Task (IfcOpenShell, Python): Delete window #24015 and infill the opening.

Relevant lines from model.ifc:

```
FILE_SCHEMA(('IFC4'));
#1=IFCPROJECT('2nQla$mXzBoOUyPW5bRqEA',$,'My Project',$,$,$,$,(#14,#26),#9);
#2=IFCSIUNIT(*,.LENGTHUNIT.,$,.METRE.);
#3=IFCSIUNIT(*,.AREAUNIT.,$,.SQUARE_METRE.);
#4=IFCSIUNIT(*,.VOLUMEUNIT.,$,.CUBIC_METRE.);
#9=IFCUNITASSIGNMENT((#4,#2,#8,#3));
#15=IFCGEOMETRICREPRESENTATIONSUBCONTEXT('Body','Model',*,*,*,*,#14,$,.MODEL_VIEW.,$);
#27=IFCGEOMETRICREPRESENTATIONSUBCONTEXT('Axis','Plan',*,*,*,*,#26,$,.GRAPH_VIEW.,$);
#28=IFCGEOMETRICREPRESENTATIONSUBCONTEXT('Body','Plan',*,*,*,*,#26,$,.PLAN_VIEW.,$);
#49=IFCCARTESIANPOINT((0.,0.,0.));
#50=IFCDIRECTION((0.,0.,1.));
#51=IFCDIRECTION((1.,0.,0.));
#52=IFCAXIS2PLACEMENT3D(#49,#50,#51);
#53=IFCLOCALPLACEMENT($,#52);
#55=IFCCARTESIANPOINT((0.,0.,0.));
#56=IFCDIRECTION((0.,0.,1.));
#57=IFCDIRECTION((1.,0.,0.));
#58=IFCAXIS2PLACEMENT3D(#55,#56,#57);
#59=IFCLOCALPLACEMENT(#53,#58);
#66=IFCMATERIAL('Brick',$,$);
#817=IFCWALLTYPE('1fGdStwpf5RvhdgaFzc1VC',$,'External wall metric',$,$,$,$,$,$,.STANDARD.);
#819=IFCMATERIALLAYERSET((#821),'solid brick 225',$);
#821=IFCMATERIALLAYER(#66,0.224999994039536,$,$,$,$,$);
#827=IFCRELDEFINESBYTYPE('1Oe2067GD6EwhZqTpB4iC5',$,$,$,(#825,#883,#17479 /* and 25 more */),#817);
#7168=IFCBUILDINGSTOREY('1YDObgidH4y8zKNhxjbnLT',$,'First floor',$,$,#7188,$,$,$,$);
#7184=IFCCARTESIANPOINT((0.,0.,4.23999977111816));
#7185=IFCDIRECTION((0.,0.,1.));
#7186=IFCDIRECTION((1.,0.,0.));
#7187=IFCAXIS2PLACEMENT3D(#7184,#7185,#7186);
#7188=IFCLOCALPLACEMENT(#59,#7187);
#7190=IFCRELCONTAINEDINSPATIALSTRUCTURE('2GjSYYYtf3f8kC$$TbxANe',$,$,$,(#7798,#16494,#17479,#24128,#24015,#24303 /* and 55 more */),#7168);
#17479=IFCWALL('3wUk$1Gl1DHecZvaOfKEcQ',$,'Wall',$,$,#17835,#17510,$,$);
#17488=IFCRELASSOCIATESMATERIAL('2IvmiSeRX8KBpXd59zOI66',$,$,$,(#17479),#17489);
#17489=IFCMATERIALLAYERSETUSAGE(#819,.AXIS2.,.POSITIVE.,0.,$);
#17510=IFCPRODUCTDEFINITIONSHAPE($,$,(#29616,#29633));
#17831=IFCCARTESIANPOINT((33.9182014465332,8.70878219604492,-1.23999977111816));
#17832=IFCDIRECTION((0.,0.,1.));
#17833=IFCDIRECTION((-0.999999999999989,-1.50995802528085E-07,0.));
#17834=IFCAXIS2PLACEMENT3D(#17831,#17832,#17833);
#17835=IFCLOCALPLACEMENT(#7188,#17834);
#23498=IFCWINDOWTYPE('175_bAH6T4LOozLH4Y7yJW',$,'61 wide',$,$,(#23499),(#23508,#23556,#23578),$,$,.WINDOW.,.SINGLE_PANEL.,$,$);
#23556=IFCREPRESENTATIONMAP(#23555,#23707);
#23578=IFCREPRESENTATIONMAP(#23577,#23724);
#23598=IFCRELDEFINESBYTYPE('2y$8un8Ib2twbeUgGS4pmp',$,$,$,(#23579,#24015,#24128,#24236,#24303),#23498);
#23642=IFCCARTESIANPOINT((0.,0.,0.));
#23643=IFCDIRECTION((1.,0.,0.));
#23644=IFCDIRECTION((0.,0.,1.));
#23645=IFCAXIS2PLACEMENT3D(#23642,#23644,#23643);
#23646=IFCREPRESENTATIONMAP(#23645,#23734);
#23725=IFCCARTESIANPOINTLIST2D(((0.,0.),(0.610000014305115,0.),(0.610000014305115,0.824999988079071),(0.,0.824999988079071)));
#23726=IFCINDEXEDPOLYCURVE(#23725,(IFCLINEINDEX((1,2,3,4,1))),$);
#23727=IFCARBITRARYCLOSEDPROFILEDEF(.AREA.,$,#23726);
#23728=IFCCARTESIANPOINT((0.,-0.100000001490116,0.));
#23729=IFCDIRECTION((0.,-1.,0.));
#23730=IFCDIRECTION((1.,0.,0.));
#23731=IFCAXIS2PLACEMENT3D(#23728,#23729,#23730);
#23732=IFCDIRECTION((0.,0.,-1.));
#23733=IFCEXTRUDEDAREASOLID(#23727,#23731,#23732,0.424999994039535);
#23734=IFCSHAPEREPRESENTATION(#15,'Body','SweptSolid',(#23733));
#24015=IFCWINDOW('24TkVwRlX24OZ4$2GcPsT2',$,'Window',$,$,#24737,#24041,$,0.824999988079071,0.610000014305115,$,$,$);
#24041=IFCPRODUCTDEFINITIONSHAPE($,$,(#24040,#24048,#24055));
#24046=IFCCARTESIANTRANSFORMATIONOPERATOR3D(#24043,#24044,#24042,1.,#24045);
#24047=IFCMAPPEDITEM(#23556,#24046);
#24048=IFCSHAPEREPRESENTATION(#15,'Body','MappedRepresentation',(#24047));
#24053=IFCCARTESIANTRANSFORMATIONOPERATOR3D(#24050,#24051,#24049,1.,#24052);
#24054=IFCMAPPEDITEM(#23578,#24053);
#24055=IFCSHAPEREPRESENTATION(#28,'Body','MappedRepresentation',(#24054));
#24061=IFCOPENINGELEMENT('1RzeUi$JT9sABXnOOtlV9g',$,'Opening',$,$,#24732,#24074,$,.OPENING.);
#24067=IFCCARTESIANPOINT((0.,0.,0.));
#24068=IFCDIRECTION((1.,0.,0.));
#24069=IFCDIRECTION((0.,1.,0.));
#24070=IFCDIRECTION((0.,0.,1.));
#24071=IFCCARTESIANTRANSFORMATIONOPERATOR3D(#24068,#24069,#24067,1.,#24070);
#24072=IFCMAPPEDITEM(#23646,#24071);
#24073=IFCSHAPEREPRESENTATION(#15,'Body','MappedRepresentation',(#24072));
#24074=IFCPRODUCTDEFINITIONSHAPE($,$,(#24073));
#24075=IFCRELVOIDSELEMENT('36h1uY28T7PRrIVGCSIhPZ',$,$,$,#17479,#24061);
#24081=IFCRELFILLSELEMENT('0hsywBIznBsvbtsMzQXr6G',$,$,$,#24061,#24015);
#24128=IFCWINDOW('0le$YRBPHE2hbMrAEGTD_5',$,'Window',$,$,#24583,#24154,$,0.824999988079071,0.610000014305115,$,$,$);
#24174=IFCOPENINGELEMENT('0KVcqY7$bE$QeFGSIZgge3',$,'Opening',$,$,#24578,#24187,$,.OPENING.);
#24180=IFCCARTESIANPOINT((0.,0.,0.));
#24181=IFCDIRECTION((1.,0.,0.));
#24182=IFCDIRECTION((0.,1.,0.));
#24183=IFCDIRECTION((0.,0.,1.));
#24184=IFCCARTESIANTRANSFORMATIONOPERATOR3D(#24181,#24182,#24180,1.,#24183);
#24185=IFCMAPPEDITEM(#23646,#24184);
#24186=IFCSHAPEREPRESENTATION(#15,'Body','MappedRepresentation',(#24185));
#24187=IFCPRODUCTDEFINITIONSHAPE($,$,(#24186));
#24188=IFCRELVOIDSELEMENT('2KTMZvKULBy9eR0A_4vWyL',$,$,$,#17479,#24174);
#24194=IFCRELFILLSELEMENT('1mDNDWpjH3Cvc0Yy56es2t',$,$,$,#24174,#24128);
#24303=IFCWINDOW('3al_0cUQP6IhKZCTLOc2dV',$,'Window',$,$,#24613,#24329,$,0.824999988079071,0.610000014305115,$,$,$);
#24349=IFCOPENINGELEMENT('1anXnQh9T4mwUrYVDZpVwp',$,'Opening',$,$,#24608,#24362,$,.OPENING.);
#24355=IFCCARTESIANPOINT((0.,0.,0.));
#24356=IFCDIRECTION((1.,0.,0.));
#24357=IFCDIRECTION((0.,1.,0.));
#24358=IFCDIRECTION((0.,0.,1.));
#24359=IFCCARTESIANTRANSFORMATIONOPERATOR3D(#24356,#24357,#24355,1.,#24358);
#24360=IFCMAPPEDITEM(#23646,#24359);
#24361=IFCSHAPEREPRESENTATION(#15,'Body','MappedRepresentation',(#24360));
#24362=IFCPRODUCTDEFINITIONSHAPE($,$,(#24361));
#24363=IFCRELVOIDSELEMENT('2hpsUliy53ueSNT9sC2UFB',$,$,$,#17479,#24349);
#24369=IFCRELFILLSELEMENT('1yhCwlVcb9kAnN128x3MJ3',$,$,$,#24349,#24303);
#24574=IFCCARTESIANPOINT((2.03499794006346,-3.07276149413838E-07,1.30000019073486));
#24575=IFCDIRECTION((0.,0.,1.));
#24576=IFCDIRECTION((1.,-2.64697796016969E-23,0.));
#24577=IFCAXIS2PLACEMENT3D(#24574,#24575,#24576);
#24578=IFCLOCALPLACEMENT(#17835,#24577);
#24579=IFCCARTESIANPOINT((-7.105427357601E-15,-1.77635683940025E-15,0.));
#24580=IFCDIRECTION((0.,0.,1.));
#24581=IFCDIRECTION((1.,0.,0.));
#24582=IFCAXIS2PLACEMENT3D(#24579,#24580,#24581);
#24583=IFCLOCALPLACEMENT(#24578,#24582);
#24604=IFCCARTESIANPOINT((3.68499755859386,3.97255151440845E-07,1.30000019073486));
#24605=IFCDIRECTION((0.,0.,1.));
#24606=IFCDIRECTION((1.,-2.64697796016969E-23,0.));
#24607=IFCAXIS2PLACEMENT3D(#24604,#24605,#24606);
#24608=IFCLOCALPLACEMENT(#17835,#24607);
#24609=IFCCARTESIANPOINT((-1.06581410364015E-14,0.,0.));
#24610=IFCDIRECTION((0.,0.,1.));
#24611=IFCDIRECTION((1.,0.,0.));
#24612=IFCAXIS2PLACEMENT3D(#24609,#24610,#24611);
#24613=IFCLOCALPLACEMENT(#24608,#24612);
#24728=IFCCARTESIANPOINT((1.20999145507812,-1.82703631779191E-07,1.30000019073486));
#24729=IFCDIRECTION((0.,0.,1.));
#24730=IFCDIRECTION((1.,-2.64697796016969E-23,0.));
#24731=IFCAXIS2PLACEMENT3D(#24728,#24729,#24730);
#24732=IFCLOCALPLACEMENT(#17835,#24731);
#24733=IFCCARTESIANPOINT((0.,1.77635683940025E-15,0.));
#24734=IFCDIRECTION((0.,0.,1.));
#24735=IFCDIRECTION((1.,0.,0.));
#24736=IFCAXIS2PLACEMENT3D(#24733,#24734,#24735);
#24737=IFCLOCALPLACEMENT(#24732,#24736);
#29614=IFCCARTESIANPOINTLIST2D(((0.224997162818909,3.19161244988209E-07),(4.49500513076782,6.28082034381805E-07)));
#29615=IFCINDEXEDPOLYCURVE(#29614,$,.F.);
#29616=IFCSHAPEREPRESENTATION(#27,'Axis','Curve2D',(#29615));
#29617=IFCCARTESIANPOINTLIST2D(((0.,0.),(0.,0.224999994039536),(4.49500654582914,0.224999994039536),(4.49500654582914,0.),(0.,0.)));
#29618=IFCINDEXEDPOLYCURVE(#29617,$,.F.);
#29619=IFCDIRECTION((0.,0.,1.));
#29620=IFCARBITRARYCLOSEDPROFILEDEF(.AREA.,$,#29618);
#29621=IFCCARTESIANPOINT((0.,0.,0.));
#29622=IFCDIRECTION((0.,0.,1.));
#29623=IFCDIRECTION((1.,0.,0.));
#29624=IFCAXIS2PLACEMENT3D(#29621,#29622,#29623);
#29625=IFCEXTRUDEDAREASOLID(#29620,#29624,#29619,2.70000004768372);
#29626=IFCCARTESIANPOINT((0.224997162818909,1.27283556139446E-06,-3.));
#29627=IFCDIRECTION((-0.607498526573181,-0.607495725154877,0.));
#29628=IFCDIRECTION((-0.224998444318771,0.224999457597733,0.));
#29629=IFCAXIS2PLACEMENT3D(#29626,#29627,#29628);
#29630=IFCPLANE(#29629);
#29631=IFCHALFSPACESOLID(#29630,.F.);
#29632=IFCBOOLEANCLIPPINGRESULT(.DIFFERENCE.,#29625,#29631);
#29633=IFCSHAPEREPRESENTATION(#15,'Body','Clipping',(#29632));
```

```python
import ifcopenshell
import ifcopenshell.api.feature
import ifcopenshell.api.root
import ifcopenshell.geom
import ifcopenshell.util.shape

model = ifcopenshell.open("model.ifc")
settings = ifcopenshell.geom.settings()


def volume(element):
    """Net volume in cubic metres, openings subtracted."""
    shape = ifcopenshell.geom.create_shape(settings, element)
    return ifcopenshell.util.shape.get_volume(shape.geometry)


window = model.by_id(24015)
opening = window.FillsVoids[0].RelatingOpeningElement
wall = opening.VoidsElements[0].RelatingBuildingElement
before = volume(wall)

ifcopenshell.api.root.remove_product(model, product=window)
ifcopenshell.api.feature.remove_feature(model, feature=opening)

after = volume(wall)

print(f"wall volume {before:.3f} -> {after:.3f} m3")

model.write("model-out.ifc")
```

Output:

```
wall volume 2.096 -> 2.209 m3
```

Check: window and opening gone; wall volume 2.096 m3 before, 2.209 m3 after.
